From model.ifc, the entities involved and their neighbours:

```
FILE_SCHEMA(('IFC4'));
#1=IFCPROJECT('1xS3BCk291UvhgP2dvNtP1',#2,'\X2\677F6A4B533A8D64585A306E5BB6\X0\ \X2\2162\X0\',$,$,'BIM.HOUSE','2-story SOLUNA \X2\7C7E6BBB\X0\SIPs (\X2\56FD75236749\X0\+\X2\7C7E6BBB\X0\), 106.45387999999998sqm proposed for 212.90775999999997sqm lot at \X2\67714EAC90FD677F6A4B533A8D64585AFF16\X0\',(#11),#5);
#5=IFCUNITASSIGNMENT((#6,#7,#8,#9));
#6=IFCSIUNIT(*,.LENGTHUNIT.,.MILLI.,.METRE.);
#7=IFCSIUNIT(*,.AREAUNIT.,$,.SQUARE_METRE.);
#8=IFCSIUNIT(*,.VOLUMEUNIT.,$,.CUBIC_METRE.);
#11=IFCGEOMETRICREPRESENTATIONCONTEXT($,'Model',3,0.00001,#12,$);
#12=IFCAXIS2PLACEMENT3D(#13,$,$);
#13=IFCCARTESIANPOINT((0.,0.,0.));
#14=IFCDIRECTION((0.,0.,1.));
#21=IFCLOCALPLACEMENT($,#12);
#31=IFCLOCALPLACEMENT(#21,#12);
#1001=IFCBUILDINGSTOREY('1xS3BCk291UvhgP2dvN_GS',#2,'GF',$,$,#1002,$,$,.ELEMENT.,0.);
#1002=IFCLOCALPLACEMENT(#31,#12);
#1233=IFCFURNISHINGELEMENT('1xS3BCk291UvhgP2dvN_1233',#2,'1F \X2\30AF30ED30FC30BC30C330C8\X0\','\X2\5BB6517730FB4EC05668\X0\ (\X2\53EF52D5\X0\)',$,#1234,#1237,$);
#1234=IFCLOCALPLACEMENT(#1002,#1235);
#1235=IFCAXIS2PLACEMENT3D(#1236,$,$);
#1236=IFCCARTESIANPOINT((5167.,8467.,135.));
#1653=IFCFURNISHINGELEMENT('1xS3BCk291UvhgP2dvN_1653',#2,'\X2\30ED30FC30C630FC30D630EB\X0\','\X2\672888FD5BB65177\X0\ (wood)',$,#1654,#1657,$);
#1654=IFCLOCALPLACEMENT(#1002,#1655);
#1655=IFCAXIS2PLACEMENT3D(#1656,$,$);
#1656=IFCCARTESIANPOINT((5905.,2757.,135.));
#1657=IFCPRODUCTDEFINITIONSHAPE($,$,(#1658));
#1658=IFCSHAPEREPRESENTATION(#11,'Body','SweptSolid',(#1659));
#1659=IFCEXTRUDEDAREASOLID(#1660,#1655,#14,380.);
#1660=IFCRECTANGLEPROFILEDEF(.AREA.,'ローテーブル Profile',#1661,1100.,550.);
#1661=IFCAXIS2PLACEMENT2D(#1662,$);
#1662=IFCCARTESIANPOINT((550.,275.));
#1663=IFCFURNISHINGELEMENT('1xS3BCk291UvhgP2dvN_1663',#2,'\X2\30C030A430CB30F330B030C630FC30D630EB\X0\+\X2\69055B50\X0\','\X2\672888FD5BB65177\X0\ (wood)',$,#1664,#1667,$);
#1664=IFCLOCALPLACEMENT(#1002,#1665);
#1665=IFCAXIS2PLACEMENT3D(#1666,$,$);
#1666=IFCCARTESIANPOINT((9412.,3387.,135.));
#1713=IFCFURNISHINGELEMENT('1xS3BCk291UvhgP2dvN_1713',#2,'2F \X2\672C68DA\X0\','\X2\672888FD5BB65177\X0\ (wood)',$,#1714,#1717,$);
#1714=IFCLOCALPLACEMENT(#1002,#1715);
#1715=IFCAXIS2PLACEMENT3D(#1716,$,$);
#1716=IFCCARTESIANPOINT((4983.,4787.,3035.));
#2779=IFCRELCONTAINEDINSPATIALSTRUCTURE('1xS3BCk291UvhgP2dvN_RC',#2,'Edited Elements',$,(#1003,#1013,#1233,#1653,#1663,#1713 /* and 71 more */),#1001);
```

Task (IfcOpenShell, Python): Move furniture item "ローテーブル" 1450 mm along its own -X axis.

```python
import ifcopenshell
import ifcopenshell.api.geometry
import ifcopenshell.util.placement
import ifcopenshell.util.unit

model = ifcopenshell.open("model.ifc")
unit_scale = ifcopenshell.util.unit.calculate_unit_scale(model)

item = model.by_guid("1xS3BCk291UvhgP2dvN_1653")
matrix = ifcopenshell.util.placement.get_local_placement(item.ObjectPlacement)
matrix[:3, 3] -= matrix[:3, 0] * 1.45 / unit_scale
ifcopenshell.api.geometry.edit_object_placement(model, product=item, matrix=matrix, is_si=False)

print(ifcopenshell.util.placement.get_local_placement(item.ObjectPlacement).round(3) + 0.0)

model.write("model-out.ifc")
```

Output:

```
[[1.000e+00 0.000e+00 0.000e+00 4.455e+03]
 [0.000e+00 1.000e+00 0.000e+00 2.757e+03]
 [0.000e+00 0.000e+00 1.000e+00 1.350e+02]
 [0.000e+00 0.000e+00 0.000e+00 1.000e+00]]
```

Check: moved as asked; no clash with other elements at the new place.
